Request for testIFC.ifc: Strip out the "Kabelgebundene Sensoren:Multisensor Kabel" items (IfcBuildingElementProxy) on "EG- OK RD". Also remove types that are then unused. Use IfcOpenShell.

First a look at what the model holds.

```python
import ifcopenshell
import ifcopenshell.util.element

model = ifcopenshell.open("testIFC.ifc")
print(model.schema)
storey = next(s for s in model.by_type("IfcBuildingStorey") if s.Name == "EG- OK RD")
proxies = [e for e in ifcopenshell.util.element.get_decomposition(storey) if e.is_a("IfcBuildingElementProxy")]
seen = {}
for e in proxies:
    element_type = ifcopenshell.util.element.get_type(e)
    name = element_type.Name if element_type not in (None, e) else None
    seen[name] = seen.get(name, 0) + 1
for name, count in sorted(seen.items(), key=str):
    print(count, "x", name)
```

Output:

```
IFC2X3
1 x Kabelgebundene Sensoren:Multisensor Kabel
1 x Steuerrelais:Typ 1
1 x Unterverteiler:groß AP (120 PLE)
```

```python
import ifcopenshell
import ifcopenshell.api.root
import ifcopenshell.util.element

model = ifcopenshell.open("testIFC.ifc")

storey = next(s for s in model.by_type("IfcBuildingStorey") if s.Name == "EG- OK RD")
proxies = [e for e in ifcopenshell.util.element.get_decomposition(storey) if e.is_a("IfcBuildingElementProxy")]
targets = [e for e in proxies if (t := ifcopenshell.util.element.get_type(e)) not in (None, e) and t.Name == "Kabelgebundene Sensoren:Multisensor Kabel"]
types = {ifcopenshell.util.element.get_type(e) for e in targets} - {None, *targets}

for e in targets:
    ifcopenshell.api.root.remove_product(model, product=e)
print(len(targets), "removed")

unused = [t for t in types if not ifcopenshell.util.element.get_types(t)]
for t in unused:
    ifcopenshell.api.root.remove_product(model, product=t)
print(len(unused), "unused types removed")

model.write("testIFC_v2.ifc")
```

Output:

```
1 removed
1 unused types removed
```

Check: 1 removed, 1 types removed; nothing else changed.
